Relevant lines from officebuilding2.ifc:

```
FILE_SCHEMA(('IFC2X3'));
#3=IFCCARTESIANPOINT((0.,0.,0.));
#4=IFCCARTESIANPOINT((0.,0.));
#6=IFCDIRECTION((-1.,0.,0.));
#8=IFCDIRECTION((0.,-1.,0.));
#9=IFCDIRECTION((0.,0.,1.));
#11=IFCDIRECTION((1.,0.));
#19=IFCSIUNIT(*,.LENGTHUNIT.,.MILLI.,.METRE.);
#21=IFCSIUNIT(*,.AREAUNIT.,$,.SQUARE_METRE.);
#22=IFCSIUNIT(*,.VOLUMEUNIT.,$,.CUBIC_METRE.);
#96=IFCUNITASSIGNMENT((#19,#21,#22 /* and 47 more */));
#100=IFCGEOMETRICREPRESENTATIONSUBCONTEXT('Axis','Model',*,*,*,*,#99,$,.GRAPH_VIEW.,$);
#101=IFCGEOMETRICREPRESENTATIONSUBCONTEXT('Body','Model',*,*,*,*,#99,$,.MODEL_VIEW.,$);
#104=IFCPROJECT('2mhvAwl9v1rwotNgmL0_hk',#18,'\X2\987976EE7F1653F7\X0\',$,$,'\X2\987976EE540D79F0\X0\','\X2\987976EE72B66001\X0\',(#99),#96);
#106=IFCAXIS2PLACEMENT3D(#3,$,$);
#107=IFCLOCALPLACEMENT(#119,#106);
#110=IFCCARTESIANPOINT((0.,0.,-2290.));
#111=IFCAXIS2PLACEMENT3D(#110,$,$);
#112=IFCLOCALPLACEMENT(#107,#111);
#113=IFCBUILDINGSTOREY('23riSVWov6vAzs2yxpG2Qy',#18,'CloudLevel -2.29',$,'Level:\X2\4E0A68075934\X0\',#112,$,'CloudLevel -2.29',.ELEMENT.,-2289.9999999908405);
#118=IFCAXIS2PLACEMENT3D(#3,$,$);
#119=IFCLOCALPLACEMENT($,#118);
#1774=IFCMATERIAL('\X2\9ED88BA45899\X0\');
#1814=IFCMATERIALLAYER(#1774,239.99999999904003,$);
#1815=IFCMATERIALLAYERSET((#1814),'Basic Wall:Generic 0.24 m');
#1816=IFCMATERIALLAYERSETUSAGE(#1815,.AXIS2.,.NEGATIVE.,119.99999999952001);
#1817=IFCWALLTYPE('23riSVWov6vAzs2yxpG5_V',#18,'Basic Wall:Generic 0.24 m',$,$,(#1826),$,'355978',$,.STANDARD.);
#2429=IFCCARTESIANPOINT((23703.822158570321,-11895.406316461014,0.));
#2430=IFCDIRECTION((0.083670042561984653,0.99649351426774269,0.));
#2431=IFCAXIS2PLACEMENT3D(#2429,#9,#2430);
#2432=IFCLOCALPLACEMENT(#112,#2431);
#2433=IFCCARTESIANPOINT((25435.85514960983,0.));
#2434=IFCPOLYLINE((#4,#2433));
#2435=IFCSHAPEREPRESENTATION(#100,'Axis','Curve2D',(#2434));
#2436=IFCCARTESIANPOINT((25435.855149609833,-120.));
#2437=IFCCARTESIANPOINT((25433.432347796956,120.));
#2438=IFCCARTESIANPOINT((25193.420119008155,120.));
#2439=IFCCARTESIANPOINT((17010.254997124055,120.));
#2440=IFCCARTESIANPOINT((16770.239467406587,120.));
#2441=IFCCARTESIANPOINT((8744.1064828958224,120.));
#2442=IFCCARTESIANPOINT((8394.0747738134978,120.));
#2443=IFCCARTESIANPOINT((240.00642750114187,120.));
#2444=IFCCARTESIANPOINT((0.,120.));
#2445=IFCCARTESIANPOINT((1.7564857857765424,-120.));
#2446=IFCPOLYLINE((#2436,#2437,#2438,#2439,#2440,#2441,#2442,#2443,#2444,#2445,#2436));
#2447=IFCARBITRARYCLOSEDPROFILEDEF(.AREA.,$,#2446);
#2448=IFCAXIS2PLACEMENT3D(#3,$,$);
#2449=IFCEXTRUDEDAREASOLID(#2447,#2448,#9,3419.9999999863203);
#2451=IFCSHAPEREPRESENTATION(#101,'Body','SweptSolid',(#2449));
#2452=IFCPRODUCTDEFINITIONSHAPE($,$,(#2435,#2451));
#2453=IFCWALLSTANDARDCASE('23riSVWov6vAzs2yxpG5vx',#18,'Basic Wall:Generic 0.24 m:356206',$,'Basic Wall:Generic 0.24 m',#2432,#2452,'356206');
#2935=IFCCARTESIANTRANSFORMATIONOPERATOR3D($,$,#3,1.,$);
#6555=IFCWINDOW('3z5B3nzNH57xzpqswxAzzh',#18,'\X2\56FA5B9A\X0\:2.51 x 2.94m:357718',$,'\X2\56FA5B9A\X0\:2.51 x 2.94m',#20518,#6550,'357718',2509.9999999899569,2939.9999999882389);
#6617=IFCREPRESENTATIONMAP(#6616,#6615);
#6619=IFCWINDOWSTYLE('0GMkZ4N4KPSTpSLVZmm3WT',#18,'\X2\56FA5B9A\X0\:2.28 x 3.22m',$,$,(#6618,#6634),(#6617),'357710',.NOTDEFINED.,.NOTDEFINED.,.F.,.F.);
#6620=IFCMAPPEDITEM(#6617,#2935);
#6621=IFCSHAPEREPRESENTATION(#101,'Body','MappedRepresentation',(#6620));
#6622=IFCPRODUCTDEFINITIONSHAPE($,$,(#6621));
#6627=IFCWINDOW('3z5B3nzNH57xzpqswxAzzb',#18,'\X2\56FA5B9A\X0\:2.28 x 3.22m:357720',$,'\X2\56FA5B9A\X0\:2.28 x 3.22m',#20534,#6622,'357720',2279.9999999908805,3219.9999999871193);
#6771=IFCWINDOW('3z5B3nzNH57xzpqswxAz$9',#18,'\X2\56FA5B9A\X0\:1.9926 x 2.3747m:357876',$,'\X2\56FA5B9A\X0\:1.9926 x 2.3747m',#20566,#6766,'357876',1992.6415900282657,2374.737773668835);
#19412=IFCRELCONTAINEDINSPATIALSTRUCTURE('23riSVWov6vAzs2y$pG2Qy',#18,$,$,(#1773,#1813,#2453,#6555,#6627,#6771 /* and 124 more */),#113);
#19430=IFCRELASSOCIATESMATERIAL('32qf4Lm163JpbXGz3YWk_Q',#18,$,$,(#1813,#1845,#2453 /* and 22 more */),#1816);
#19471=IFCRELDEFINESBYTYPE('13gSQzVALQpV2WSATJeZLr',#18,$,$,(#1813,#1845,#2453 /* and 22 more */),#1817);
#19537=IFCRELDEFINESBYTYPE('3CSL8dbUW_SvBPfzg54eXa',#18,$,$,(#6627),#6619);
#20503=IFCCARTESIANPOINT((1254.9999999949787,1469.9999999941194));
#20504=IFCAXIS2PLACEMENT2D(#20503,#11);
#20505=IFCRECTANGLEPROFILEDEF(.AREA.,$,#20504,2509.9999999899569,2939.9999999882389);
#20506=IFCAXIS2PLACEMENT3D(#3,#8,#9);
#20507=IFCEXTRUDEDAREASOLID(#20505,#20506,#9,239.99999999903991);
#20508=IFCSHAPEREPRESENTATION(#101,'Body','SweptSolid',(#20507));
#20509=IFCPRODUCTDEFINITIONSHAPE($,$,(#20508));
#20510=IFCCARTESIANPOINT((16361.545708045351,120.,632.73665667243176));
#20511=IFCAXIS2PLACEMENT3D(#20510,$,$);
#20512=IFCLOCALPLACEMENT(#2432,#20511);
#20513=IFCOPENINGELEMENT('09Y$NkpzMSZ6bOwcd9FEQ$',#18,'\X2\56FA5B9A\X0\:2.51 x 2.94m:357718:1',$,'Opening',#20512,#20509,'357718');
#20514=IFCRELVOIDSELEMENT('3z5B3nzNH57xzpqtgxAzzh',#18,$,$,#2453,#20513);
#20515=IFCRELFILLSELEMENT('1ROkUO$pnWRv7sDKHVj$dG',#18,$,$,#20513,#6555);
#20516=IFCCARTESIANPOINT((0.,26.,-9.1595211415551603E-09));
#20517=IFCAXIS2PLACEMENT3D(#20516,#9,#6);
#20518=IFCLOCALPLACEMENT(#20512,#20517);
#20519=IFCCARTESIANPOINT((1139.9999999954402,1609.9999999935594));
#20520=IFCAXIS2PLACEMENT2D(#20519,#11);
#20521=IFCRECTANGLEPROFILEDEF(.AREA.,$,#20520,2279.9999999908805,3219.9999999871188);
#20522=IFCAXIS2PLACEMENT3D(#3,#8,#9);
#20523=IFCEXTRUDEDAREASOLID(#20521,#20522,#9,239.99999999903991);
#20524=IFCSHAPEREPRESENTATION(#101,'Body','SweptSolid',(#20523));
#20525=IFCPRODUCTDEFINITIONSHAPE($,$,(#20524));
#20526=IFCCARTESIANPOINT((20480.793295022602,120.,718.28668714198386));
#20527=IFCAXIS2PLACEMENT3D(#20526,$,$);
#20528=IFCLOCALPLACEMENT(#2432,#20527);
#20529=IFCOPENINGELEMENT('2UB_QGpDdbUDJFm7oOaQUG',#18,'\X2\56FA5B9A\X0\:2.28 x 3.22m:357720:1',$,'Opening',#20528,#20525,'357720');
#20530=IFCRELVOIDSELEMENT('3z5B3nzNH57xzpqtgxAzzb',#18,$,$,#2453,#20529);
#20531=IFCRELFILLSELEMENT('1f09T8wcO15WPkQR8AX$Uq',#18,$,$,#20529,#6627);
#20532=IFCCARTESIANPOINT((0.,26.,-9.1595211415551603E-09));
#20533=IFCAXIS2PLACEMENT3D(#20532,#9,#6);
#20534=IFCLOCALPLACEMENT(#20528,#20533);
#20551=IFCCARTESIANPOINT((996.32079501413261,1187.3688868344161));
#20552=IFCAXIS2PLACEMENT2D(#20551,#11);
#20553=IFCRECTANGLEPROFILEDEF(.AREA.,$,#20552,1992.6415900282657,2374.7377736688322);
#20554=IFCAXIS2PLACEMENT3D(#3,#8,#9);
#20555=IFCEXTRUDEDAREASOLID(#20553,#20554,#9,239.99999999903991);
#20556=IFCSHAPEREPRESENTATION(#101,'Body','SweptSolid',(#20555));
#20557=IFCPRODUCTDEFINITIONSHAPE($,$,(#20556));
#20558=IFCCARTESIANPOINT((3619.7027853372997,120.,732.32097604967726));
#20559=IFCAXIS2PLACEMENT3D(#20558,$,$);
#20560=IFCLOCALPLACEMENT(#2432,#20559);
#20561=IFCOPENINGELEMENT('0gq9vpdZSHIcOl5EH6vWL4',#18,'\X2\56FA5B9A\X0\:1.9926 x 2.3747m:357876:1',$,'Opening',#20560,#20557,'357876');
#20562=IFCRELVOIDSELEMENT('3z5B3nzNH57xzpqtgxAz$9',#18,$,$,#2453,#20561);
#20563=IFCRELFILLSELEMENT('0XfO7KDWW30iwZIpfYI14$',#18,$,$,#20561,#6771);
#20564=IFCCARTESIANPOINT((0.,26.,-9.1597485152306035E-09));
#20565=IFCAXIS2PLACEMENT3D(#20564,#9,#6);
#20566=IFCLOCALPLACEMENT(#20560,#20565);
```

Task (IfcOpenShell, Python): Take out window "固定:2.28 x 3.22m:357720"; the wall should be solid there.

```python
import ifcopenshell
import ifcopenshell.api.feature
import ifcopenshell.api.root
import ifcopenshell.geom
import ifcopenshell.util.shape

model = ifcopenshell.open("officebuilding2.ifc")
settings = ifcopenshell.geom.settings()


def volume(element):
    """Net volume in cubic metres, openings subtracted."""
    shape = ifcopenshell.geom.create_shape(settings, element)
    return ifcopenshell.util.shape.get_volume(shape.geometry)


window = model.by_guid("3z5B3nzNH57xzpqswxAzzb")
opening = window.FillsVoids[0].RelatingOpeningElement
wall = opening.VoidsElements[0].RelatingBuildingElement
before = volume(wall)

ifcopenshell.api.root.remove_product(model, product=window)
ifcopenshell.api.feature.remove_feature(model, feature=opening)

after = volume(wall)

print(f"wall volume {before:.3f} -> {after:.3f} m3")

model.write("officebuilding2_v2.ifc")
```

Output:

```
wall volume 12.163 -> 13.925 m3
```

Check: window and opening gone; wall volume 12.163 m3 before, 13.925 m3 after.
